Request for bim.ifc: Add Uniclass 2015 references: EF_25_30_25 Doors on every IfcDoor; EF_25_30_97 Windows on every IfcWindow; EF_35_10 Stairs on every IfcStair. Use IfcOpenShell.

First a look at what the model holds.

```python
import ifcopenshell

model = ifcopenshell.open("bim.ifc")
print(model.schema)
print("classifications:", [c.Name for c in model.by_type("IfcClassification")])
for ifc_class in ("IfcDoor", "IfcRoof", "IfcStair", "IfcWall", "IfcWindow"):
    print(ifc_class, len(model.by_type(ifc_class)))
```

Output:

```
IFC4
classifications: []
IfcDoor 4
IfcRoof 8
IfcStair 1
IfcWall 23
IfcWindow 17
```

```python
import ifcopenshell
import ifcopenshell.api.classification

model = ifcopenshell.open("bim.ifc")

system = ifcopenshell.api.classification.add_classification(model, classification="Uniclass 2015")

codes = {
    "IfcDoor": ("EF_25_30_25", "Doors"),
    "IfcWindow": ("EF_25_30_97", "Windows"),
    "IfcStair": ("EF_35_10", "Stairs"),
}
for ifc_class, (code, name) in codes.items():
    products = model.by_type(ifc_class)
    ifcopenshell.api.classification.add_reference(
        model, products=products, classification=system, identification=code, name=name
    )
    print(code, len(products))

model.write("bim_rev.ifc")
```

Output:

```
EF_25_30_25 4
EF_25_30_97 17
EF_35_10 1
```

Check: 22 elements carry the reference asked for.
